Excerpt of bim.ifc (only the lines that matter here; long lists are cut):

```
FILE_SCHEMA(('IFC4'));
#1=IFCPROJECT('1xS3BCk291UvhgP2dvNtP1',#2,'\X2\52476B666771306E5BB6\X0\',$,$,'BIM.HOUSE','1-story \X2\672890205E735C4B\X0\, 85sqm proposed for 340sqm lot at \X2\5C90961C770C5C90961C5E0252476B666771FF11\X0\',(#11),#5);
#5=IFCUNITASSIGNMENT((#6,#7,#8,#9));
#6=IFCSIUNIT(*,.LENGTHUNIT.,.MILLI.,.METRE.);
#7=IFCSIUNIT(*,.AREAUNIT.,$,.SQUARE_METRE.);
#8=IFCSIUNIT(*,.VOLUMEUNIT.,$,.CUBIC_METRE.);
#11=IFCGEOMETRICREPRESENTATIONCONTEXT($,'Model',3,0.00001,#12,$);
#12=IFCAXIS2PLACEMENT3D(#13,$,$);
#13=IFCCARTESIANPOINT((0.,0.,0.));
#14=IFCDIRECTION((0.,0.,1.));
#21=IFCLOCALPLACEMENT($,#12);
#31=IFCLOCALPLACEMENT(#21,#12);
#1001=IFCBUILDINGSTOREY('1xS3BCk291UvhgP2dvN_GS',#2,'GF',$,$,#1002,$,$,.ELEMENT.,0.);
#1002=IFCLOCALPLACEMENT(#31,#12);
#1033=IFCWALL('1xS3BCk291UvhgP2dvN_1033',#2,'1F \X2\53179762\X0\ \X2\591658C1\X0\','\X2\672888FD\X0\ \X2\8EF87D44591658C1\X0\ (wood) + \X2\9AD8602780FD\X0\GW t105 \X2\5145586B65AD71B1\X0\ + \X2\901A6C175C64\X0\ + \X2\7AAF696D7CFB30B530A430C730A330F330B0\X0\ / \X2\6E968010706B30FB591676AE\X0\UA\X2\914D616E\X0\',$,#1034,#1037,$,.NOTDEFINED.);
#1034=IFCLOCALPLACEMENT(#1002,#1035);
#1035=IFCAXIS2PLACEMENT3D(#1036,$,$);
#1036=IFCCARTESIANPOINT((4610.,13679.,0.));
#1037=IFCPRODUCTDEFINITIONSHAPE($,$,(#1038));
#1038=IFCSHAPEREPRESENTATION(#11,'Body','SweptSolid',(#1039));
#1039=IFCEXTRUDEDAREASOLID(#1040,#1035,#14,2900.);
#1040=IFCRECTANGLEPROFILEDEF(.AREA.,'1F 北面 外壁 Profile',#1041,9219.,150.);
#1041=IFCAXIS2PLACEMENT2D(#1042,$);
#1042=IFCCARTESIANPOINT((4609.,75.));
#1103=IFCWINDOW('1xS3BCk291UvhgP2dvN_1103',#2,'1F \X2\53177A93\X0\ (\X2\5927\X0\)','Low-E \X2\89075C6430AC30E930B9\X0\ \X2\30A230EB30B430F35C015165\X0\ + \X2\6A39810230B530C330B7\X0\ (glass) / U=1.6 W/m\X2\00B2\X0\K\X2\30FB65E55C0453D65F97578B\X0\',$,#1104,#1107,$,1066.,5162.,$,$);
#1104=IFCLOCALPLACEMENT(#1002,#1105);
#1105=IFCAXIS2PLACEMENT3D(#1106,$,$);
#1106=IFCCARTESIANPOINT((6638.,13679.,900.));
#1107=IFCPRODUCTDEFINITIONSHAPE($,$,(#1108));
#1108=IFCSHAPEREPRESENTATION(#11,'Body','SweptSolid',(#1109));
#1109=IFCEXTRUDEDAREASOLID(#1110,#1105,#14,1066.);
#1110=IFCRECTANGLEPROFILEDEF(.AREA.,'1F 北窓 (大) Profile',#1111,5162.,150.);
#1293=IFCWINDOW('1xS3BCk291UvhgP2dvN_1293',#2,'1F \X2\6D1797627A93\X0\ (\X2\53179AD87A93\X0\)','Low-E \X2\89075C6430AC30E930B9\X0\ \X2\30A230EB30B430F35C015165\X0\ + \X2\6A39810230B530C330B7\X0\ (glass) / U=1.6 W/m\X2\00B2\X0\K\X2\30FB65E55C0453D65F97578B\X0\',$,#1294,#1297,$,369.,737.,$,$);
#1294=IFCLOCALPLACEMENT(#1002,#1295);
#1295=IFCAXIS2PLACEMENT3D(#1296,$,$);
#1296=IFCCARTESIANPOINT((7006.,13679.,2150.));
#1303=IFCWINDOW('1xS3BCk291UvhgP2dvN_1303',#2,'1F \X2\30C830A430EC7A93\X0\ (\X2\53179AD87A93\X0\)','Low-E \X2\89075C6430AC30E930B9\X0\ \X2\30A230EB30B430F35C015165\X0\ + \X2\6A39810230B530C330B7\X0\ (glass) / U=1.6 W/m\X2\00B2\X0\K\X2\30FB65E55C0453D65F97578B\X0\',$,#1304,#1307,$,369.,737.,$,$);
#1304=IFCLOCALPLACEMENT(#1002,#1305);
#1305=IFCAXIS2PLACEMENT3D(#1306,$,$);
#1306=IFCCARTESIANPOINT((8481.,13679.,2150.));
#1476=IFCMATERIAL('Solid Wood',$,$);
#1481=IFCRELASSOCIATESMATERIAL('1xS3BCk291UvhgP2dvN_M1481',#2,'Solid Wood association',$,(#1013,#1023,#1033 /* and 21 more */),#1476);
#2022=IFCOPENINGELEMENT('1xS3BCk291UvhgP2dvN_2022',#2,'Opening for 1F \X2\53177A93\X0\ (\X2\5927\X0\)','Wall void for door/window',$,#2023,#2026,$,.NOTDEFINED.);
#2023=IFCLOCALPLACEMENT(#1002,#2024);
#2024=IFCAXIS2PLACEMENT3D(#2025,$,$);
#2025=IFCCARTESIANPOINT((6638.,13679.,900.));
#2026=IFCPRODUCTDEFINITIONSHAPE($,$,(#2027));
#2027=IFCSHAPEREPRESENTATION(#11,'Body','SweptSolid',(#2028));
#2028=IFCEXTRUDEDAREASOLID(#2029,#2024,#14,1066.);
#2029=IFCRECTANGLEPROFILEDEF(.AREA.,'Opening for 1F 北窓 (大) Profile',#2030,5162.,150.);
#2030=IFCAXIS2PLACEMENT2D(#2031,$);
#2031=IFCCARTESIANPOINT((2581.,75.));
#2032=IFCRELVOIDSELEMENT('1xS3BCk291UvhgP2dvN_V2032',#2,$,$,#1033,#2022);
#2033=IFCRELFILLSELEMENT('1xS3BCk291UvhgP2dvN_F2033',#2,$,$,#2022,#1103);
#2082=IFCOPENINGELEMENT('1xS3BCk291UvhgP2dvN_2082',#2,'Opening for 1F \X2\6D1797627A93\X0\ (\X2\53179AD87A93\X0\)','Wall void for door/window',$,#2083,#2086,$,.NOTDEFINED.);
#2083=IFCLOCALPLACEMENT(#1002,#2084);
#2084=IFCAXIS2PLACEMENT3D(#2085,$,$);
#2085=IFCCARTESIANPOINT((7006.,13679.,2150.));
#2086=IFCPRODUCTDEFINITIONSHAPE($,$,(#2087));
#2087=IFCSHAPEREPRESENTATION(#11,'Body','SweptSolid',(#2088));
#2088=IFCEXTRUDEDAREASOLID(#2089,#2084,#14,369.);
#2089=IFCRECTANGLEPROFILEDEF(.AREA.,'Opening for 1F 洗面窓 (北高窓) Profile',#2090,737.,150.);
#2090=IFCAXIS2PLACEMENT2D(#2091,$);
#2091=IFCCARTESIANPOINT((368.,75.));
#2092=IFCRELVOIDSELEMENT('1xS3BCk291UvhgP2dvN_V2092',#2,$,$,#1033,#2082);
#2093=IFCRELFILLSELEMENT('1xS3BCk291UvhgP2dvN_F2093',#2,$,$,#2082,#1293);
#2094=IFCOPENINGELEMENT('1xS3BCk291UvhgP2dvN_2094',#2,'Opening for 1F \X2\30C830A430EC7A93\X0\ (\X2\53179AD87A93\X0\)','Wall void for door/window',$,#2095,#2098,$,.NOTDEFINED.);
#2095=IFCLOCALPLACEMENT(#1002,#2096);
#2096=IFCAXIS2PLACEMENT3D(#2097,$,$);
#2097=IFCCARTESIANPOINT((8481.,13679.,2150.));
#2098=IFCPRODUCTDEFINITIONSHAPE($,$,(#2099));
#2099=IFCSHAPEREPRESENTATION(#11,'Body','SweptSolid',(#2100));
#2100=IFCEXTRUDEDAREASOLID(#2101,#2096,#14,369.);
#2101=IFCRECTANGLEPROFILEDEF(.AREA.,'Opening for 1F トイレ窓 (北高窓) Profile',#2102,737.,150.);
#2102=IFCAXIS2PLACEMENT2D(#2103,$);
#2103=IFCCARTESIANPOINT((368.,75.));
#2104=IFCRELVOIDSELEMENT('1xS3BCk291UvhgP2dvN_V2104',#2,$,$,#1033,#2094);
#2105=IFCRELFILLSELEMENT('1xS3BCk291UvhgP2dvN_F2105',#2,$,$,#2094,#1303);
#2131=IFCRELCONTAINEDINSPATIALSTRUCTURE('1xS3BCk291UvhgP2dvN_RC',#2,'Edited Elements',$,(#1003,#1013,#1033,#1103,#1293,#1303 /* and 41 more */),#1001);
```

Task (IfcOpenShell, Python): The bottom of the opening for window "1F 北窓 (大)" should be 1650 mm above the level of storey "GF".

```python
import numpy as np
import ifcopenshell
import ifcopenshell.api.geometry
import ifcopenshell.geom
import ifcopenshell.util.element
import ifcopenshell.util.placement
import ifcopenshell.util.shape
import ifcopenshell.util.unit

model = ifcopenshell.open("bim.ifc")
unit_scale = ifcopenshell.util.unit.calculate_unit_scale(model)

window = model.by_guid("1xS3BCk291UvhgP2dvN_1103")
opening = window.FillsVoids[0].RelatingOpeningElement
storey = ifcopenshell.util.element.get_container(window, ifc_class="IfcBuildingStorey")
level = ifcopenshell.util.placement.get_local_placement(storey.ObjectPlacement)[2, 3]

# The opening's origin need not be at the sill, so measure its lowest point.
shape = ifcopenshell.geom.create_shape(ifcopenshell.geom.settings(), opening)
bottom = ifcopenshell.util.shape.get_shape_bottom_elevation(shape, shape.geometry) / unit_scale
dz = level + 1.65 / unit_scale - bottom

shift = np.array([0.0, 0.0, dz])
# The window is not placed relative to its opening, so move both.
for product in (opening, window):
    matrix = ifcopenshell.util.placement.get_local_placement(product.ObjectPlacement)
    matrix[:3, 3] += shift
    ifcopenshell.api.geometry.edit_object_placement(model, product=product, matrix=matrix, is_si=False)

print(f"moved by {dz * unit_scale:+.3f} m")

model.write("bim_v2.ifc")
```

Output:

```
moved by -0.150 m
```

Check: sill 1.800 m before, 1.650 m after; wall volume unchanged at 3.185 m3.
